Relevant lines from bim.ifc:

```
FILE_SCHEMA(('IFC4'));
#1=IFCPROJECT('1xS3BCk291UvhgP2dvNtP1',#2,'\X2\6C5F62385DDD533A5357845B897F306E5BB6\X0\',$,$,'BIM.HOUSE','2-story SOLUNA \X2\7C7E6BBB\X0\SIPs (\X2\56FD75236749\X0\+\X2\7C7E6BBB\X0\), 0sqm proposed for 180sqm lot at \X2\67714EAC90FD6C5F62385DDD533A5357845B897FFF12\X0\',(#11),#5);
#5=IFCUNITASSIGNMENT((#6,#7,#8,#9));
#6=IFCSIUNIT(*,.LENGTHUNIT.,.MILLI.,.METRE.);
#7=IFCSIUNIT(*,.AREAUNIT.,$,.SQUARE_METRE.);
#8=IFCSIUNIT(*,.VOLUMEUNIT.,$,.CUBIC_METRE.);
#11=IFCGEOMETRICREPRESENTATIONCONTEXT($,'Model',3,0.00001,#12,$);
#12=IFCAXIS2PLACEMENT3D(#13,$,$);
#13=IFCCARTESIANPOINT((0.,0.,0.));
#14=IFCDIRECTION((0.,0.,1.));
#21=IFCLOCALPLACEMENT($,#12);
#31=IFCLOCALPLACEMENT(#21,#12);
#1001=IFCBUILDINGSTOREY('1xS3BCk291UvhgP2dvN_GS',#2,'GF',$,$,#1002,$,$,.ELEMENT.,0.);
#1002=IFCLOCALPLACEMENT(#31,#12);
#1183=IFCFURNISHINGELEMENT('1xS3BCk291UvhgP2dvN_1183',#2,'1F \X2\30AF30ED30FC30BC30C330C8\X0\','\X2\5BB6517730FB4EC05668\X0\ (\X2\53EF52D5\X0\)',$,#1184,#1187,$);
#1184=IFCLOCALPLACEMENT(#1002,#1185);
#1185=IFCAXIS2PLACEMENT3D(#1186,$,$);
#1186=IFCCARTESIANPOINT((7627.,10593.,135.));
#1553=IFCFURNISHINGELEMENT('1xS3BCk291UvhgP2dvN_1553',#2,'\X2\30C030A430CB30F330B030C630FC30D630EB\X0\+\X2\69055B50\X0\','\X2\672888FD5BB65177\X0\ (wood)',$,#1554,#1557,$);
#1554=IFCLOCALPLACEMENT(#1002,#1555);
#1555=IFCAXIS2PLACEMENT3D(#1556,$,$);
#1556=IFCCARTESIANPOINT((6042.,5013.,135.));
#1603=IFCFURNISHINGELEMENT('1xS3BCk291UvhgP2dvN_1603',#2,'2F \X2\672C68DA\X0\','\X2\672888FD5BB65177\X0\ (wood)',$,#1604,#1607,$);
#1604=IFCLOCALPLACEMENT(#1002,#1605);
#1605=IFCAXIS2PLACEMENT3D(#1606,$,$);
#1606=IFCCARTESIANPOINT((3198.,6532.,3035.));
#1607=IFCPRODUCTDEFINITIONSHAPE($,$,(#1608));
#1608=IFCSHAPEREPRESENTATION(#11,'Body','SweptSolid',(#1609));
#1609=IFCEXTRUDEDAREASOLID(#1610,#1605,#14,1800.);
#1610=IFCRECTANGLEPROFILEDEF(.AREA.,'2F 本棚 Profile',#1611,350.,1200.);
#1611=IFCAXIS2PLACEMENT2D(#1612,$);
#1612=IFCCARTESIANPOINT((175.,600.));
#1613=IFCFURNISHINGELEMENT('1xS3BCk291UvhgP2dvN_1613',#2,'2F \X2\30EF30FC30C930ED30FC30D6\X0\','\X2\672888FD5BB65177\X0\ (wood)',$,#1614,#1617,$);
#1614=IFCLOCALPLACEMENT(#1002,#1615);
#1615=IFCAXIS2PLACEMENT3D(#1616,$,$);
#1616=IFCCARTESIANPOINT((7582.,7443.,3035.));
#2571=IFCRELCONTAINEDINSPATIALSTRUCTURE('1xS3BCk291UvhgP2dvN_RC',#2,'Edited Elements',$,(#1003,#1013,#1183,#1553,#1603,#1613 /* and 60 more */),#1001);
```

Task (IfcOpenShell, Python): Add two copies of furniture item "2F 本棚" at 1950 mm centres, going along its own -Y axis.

```python
import ifcopenshell
import ifcopenshell.api.geometry
import ifcopenshell.api.root
import ifcopenshell.util.element
import ifcopenshell.util.placement

model = ifcopenshell.open("bim.ifc")


def reuse_history(source, copy):
    """copy_class also copies each property set's owner history, people and application; keep the originals."""
    for rel in copy.IsDefinedBy:
        if rel.is_a("IfcRelDefinesByProperties") and (history := rel.RelatingPropertyDefinition.OwnerHistory):
            rel.RelatingPropertyDefinition.OwnerHistory = source.OwnerHistory
            ifcopenshell.util.element.remove_deep2(model, history)


source = model.by_guid("1xS3BCk291UvhgP2dvN_1603")
base = ifcopenshell.util.placement.get_local_placement(source.ObjectPlacement)
step = -base[:3, 1] * 1950.0

for i in range(1, 3):
    copy = ifcopenshell.api.root.copy_class(model, product=source)
    copy.Representation = ifcopenshell.util.element.copy_deep(
        model, source.Representation, exclude=["IfcGeometricRepresentationContext", "IfcRepresentationMap"]
    )
    reuse_history(source, copy)
    matrix = base.copy()
    matrix[:3, 3] += i * step
    print("added at", matrix[:3, 3].round(3) + 0.0)
    ifcopenshell.api.geometry.edit_object_placement(model, product=copy, matrix=matrix, is_si=False)

model.write("bim-out.ifc")
```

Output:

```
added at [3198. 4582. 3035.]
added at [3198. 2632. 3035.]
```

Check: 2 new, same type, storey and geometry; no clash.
